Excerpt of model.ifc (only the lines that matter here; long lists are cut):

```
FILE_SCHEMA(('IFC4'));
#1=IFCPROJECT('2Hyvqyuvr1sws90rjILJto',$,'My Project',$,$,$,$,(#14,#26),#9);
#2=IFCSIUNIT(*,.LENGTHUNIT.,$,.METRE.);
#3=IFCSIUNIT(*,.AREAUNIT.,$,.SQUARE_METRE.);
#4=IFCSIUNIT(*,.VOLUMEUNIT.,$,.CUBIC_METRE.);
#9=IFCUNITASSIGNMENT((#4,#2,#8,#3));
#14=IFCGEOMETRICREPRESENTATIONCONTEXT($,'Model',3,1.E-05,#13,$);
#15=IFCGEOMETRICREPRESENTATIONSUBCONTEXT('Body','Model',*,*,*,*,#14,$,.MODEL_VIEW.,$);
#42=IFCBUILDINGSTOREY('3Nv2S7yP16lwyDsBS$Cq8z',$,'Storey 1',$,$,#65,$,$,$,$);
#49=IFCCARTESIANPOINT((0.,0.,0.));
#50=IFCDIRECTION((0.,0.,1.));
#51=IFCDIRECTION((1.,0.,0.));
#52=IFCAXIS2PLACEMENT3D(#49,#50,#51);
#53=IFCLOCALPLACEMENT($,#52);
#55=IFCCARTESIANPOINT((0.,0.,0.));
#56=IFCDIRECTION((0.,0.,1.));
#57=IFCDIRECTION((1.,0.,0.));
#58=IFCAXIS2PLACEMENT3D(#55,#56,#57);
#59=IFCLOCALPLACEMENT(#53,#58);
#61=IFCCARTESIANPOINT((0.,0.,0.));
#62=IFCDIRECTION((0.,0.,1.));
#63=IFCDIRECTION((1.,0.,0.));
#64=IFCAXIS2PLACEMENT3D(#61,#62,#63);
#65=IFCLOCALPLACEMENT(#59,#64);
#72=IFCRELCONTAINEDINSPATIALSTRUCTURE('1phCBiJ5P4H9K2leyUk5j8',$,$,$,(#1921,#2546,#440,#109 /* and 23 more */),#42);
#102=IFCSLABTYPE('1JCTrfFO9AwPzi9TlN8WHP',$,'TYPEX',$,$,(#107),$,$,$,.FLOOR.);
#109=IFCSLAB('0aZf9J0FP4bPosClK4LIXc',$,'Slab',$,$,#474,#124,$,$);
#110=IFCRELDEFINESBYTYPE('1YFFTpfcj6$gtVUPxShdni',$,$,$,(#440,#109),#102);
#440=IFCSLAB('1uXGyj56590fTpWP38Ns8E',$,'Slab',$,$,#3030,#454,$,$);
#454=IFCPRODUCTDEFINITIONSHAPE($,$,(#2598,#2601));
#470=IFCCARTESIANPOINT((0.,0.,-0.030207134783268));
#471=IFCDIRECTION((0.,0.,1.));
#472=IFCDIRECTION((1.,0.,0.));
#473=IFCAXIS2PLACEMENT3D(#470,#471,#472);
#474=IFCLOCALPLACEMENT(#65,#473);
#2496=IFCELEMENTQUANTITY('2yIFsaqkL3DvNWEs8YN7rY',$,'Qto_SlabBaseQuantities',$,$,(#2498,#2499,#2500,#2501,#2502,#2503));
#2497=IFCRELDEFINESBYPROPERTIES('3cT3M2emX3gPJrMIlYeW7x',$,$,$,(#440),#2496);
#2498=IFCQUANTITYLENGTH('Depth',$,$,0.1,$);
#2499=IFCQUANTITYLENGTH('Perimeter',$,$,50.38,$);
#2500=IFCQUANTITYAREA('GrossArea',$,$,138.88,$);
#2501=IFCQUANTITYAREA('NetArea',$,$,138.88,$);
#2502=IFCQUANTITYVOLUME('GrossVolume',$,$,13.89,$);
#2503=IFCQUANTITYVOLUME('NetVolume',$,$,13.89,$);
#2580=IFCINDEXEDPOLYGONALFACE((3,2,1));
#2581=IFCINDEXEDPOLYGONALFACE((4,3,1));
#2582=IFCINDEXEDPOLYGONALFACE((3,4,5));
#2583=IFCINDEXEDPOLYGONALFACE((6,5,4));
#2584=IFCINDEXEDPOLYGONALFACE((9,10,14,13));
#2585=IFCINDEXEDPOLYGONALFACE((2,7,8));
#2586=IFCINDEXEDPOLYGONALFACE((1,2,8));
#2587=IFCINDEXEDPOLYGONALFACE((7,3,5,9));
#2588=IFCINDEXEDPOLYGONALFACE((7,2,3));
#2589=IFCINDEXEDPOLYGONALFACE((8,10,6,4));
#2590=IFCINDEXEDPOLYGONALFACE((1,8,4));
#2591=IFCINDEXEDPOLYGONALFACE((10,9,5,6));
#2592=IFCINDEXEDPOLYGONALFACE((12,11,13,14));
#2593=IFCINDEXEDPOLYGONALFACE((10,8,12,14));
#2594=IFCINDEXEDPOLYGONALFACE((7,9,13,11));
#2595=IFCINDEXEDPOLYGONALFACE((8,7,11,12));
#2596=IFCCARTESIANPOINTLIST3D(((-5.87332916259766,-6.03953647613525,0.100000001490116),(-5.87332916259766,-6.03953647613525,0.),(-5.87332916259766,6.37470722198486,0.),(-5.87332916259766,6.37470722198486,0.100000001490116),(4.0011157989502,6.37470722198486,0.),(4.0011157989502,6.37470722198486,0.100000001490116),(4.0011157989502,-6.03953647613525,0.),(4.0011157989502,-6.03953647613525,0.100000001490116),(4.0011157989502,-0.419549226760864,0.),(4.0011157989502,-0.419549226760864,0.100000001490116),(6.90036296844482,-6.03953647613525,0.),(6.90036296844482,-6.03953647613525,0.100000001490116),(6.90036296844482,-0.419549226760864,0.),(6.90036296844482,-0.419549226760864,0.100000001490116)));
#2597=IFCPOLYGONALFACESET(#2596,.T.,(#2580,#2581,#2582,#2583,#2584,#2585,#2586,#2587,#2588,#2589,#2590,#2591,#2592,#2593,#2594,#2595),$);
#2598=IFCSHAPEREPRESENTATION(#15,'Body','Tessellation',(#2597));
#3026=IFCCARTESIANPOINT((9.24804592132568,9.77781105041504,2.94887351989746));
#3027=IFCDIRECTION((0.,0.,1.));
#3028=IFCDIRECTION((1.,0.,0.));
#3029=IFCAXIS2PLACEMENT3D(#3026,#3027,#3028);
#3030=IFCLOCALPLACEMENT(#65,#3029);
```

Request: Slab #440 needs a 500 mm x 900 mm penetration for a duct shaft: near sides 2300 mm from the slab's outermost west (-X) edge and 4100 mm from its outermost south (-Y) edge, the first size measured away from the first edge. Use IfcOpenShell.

```python
import numpy as np
import ifcopenshell
import ifcopenshell.api.feature
import ifcopenshell.api.geometry
import ifcopenshell.api.pset
import ifcopenshell.api.root
import ifcopenshell.geom
import ifcopenshell.util.element
import ifcopenshell.util.placement
import ifcopenshell.util.representation
import ifcopenshell.util.shape
import ifcopenshell.util.unit

model = ifcopenshell.open("model.ifc")
unit_scale = ifcopenshell.util.unit.calculate_unit_scale(model)
area_scale = ifcopenshell.util.unit.calculate_unit_scale(model, "AREAUNIT")
volume_scale = ifcopenshell.util.unit.calculate_unit_scale(model, "VOLUMEUNIT")
settings = ifcopenshell.geom.settings()


def volume(element):
    """Net volume in cubic metres, openings subtracted."""
    shape = ifcopenshell.geom.create_shape(settings, element)
    return ifcopenshell.util.shape.get_volume(shape.geometry)


slab = model.by_guid("1uXGyj56590fTpWP38Ns8E")
before = volume(slab)

# Extent in the slab's own axes, in metres. The edges named are its -X and -Y sides.
slab_shape = ifcopenshell.geom.create_shape(settings, slab)
vertices = ifcopenshell.util.shape.get_vertices(slab_shape.geometry)
x_min, y_min, bottom = vertices.min(axis=0)
top = vertices[:, 2].max()

opening = ifcopenshell.api.root.create_entity(model, ifc_class="IfcOpeningElement", name="Duct shaft opening", predefined_type="OPENING")
context = ifcopenshell.util.representation.get_context(model, "Model", "Body", "MODEL_VIEW")
width, depth = 0.5, 0.9
outline = [(0.0, 0.0), (width, 0.0), (width, depth), (0.0, depth), (0.0, 0.0)]
# Overshoot both faces by 50 mm so the cut is clean.
shape = ifcopenshell.api.geometry.add_slab_representation(
    model, context=context, depth=top - bottom + 0.1, polyline=outline
)
ifcopenshell.api.geometry.assign_representation(model, product=opening, representation=shape)

matrix = ifcopenshell.util.placement.get_local_placement(slab.ObjectPlacement)
matrix[:, 3] = matrix @ np.append(np.array([x_min + 2.3, y_min + 4.1, bottom - 0.05]) / unit_scale, 1.0)
ifcopenshell.api.geometry.edit_object_placement(model, product=opening, matrix=matrix, is_si=False)
ifcopenshell.api.feature.add_feature(model, feature=opening, element=slab)

after = volume(slab)

# Update the slab's stored quantities.
qto = model.by_id(ifcopenshell.util.element.get_pset(slab, "Qto_SlabBaseQuantities", should_inherit=False)["id"])
ifcopenshell.api.pset.edit_qto(model, qto=qto, properties={
    "NetArea": after / (top - bottom) / area_scale,
    "NetVolume": after / volume_scale,
})

print(f"slab volume {before:.3f} -> {after:.3f} m3")

model.write("model_v2.ifc")
```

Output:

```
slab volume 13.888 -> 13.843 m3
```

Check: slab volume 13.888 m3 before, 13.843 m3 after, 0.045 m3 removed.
